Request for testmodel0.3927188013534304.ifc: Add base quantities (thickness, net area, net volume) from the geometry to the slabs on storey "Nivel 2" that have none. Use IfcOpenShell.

First a look at what the model holds.

```python
import ifcopenshell
import ifcopenshell.util.element
import ifcopenshell.util.unit

model = ifcopenshell.open("testmodel0.3927188013534304.ifc")
print(model.schema)
for unit_type in ("LENGTHUNIT", "AREAUNIT", "VOLUMEUNIT"):
    print(unit_type, ifcopenshell.util.unit.calculate_unit_scale(model, unit_type))
storey = next(s for s in model.by_type("IfcBuildingStorey") if s.Name == "Nivel 2")
slabs = [e for e in ifcopenshell.util.element.get_decomposition(storey) if e.is_a("IfcSlab")]
for e in sorted(slabs, key=lambda e: e.id()):
    print(e.id(), e.is_a(), e.Name, list(ifcopenshell.util.element.get_psets(e, qtos_only=True)), sep=" | ")
```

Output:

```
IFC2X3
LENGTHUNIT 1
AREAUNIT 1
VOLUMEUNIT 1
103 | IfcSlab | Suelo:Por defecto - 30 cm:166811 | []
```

```python
import ifcopenshell
import ifcopenshell.api.pset
import ifcopenshell.geom
import ifcopenshell.util.element
import ifcopenshell.util.shape
import ifcopenshell.util.unit

model = ifcopenshell.open("testmodel0.3927188013534304.ifc")
unit_scale = ifcopenshell.util.unit.calculate_unit_scale(model)
area_scale = ifcopenshell.util.unit.calculate_unit_scale(model, "AREAUNIT")
volume_scale = ifcopenshell.util.unit.calculate_unit_scale(model, "VOLUMEUNIT")
settings = ifcopenshell.geom.settings()

storey = next(s for s in model.by_type("IfcBuildingStorey") if s.Name == "Nivel 2")
slabs = [e for e in ifcopenshell.util.element.get_decomposition(storey) if e.is_a("IfcSlab")]

for e in sorted(slabs, key=lambda e: e.id()):
    if ifcopenshell.util.element.get_psets(e, qtos_only=True, should_inherit=False):
        continue
    # Geometry comes back in metres, in the element's own axes.
    shape = ifcopenshell.geom.create_shape(settings, e)
    values = {
        "Width": ifcopenshell.util.shape.get_z(shape.geometry) / unit_scale,
        "NetArea": ifcopenshell.util.shape.get_footprint_area(shape.geometry) / area_scale,
        "NetVolume": ifcopenshell.util.shape.get_volume(shape.geometry) / volume_scale,
    }
    qto = ifcopenshell.api.pset.add_qto(model, product=e, name="BaseQuantities")
    ifcopenshell.api.pset.edit_qto(model, qto=qto, properties=values)
    print(e.id(), {k: round(v, 3) for k, v in values.items()})

model.write("testmodel0.3927188013534304_v2.ifc")
```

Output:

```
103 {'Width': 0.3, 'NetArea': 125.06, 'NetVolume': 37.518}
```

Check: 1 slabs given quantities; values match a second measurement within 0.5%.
